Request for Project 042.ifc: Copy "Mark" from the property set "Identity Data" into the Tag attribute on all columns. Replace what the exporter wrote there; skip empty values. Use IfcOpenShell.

First a look at what the model holds.

```python
import ifcopenshell
import ifcopenshell.util.element

model = ifcopenshell.open("Project 042.ifc")
print(model.schema)
columns = model.by_type("IfcColumn")
print(len(columns), "columns")
for e in columns[:8]:
    source = ifcopenshell.util.element.get_pset(e, "Identity Data", "Mark")
    target = e.Tag
    print(e.id(), repr(source), repr(target), sep=" | ")
```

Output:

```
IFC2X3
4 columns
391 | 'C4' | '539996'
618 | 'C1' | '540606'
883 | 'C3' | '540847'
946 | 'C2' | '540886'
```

```python
import ifcopenshell
import ifcopenshell.util.element

model = ifcopenshell.open("Project 042.ifc")

count = 0
for e in model.by_type("IfcColumn"):
    value = ifcopenshell.util.element.get_pset(e, "Identity Data", "Mark")
    current = e.Tag
    if not value or not value.strip() or current == value:
        continue
    e.Tag = value
    count += 1

print(count, "columns updated")

model.write("Project 042_rev.ifc")
```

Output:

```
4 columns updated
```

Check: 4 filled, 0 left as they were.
